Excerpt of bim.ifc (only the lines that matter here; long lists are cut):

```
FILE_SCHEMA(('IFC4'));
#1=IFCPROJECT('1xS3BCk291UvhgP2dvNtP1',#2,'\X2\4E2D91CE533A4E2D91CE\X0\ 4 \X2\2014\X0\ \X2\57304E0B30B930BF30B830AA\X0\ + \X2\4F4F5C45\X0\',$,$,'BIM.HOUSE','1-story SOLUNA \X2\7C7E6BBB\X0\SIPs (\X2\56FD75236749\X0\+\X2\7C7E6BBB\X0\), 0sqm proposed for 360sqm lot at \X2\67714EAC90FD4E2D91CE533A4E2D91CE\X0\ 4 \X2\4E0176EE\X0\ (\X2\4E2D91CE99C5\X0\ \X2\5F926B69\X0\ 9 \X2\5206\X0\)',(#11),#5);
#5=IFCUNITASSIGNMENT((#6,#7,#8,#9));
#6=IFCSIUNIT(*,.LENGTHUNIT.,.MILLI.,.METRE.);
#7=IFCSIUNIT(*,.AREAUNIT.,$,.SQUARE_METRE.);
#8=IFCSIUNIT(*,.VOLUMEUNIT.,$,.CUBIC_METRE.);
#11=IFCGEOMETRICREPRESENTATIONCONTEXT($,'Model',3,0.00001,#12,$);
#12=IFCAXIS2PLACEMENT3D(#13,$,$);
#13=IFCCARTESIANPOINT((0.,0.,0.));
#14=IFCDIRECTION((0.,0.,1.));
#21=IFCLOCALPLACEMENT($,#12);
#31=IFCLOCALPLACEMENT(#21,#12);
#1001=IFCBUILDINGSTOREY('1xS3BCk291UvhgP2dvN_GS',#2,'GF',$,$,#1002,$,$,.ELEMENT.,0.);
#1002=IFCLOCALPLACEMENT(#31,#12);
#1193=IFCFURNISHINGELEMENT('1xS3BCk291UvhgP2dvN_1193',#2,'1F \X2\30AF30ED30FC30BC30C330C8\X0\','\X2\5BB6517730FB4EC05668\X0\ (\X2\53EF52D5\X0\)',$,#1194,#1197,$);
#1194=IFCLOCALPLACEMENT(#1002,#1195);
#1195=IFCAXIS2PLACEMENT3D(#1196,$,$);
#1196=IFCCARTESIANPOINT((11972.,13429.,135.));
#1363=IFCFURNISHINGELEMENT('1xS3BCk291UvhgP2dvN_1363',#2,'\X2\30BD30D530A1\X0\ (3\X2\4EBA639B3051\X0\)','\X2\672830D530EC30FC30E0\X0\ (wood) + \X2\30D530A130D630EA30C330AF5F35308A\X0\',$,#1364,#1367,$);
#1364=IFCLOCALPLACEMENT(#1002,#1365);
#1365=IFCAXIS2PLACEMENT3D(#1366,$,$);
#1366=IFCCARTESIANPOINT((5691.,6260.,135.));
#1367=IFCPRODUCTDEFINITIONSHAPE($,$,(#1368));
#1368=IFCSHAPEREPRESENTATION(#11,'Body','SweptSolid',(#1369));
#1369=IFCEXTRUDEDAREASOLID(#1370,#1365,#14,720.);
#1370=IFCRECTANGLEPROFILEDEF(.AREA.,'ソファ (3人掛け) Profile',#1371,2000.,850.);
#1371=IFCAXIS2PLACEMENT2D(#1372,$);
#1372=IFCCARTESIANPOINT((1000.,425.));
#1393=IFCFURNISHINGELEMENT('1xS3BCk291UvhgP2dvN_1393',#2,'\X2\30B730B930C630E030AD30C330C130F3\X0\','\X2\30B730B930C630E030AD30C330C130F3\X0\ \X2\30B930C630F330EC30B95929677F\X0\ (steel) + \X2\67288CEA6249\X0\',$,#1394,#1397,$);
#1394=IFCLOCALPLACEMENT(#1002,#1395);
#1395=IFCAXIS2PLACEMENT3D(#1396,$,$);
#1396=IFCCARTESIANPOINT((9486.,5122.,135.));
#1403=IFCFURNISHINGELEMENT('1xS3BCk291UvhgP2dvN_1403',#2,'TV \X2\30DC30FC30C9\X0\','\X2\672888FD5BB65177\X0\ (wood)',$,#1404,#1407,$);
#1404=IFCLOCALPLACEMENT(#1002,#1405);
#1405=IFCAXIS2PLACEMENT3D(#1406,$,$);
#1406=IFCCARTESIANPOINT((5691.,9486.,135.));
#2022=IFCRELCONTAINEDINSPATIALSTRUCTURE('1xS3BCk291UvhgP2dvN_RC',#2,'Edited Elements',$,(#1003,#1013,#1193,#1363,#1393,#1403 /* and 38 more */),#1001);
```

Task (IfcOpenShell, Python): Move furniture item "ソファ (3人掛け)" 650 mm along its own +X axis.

```python
import ifcopenshell
import ifcopenshell.api.geometry
import ifcopenshell.util.placement
import ifcopenshell.util.unit

model = ifcopenshell.open("bim.ifc")
unit_scale = ifcopenshell.util.unit.calculate_unit_scale(model)

item = model.by_id(1363)
matrix = ifcopenshell.util.placement.get_local_placement(item.ObjectPlacement)
matrix[:3, 3] += matrix[:3, 0] * 0.65 / unit_scale
ifcopenshell.api.geometry.edit_object_placement(model, product=item, matrix=matrix, is_si=False)

print(ifcopenshell.util.placement.get_local_placement(item.ObjectPlacement).round(3) + 0.0)

model.write("bim_edited.ifc")
```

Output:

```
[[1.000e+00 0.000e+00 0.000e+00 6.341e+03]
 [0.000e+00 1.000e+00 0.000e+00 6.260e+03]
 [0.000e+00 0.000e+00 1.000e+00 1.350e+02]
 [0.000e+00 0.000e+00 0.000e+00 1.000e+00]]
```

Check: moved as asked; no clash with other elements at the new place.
